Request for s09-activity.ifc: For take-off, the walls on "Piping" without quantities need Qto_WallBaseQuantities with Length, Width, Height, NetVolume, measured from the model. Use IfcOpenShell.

First a look at what the model holds.

```python
import ifcopenshell
import ifcopenshell.util.element
import ifcopenshell.util.unit

model = ifcopenshell.open("s09-activity.ifc")
print(model.schema)
for unit_type in ("LENGTHUNIT", "AREAUNIT", "VOLUMEUNIT"):
    print(unit_type, ifcopenshell.util.unit.calculate_unit_scale(model, unit_type))
storey = next(s for s in model.by_type("IfcBuildingStorey") if s.Name == "Piping")
walls = [e for e in ifcopenshell.util.element.get_decomposition(storey) if e.is_a("IfcWall")]
for e in sorted(walls, key=lambda e: e.id()):
    print(e.id(), e.is_a(), e.Name, list(ifcopenshell.util.element.get_psets(e, qtos_only=True)), sep=" | ")
```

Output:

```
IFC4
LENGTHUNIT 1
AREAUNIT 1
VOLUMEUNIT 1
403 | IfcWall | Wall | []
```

```python
import ifcopenshell
import ifcopenshell.api.pset
import ifcopenshell.geom
import ifcopenshell.util.element
import ifcopenshell.util.shape
import ifcopenshell.util.unit

model = ifcopenshell.open("s09-activity.ifc")
unit_scale = ifcopenshell.util.unit.calculate_unit_scale(model)
volume_scale = ifcopenshell.util.unit.calculate_unit_scale(model, "VOLUMEUNIT")
settings = ifcopenshell.geom.settings()

storey = next(s for s in model.by_type("IfcBuildingStorey") if s.Name == "Piping")
walls = [e for e in ifcopenshell.util.element.get_decomposition(storey) if e.is_a("IfcWall")]

for e in sorted(walls, key=lambda e: e.id()):
    if ifcopenshell.util.element.get_psets(e, qtos_only=True, should_inherit=False):
        continue
    # Geometry comes back in metres, in the element's own axes.
    shape = ifcopenshell.geom.create_shape(settings, e)
    values = {
        "Length": ifcopenshell.util.shape.get_x(shape.geometry) / unit_scale,
        "Width": ifcopenshell.util.shape.get_y(shape.geometry) / unit_scale,
        "Height": ifcopenshell.util.shape.get_z(shape.geometry) / unit_scale,
        "NetVolume": ifcopenshell.util.shape.get_volume(shape.geometry) / volume_scale,
    }
    qto = ifcopenshell.api.pset.add_qto(model, product=e, name="Qto_WallBaseQuantities")
    ifcopenshell.api.pset.edit_qto(model, qto=qto, properties=values)
    print(e.id(), {k: round(v, 3) for k, v in values.items()})

model.write("s09-activity-out.ifc")
```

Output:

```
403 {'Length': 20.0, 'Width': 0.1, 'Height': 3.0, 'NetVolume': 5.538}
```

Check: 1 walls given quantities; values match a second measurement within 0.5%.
